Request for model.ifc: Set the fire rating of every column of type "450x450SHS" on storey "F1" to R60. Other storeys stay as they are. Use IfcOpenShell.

First a look at what the model holds.

```python
import ifcopenshell
import ifcopenshell.util.element

model = ifcopenshell.open("model.ifc")
print(model.schema)
storey = next(s for s in model.by_type("IfcBuildingStorey") if s.Name == "F1")
columns = [e for e in ifcopenshell.util.element.get_decomposition(storey) if e.is_a("IfcColumn")]
seen = {}
for e in columns:
    element_type = ifcopenshell.util.element.get_type(e)
    key = (element_type.Name if element_type != e and element_type else None, ifcopenshell.util.element.get_pset(e, "Pset_ColumnCommon", "FireRating"))
    seen[key] = seen.get(key, 0) + 1
for (name, value), count in sorted(seen.items(), key=str):
    print(count, "x", name, "|", value)
```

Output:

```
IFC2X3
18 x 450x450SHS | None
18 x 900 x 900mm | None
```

```python
import ifcopenshell
import ifcopenshell.api.pset
import ifcopenshell.util.element

model = ifcopenshell.open("model.ifc")

storey = next(s for s in model.by_type("IfcBuildingStorey") if s.Name == "F1")
columns = [e for e in ifcopenshell.util.element.get_decomposition(storey) if e.is_a("IfcColumn")]

count = 0
for e in columns:
    element_type = ifcopenshell.util.element.get_type(e)
    if element_type in (None, e) or element_type.Name != "450x450SHS":
        continue
    # add_pset returns the element's existing set when there is one.
    pset = ifcopenshell.api.pset.add_pset(model, product=e, name="Pset_ColumnCommon")
    ifcopenshell.api.pset.edit_pset(model, pset=pset, properties={"FireRating": "R60"})
    count += 1

print(count, "columns updated")

model.write("model-out.ifc")
```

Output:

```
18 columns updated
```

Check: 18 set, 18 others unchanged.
